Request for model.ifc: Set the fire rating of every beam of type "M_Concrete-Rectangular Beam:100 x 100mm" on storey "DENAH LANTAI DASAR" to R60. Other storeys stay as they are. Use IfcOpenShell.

First a look at what the model holds.

```python
import ifcopenshell
import ifcopenshell.util.element

model = ifcopenshell.open("model.ifc")
print(model.schema)
storey = next(s for s in model.by_type("IfcBuildingStorey") if s.Name == "DENAH LANTAI DASAR")
beams = [e for e in ifcopenshell.util.element.get_decomposition(storey) if e.is_a("IfcBeam")]
seen = {}
for e in beams:
    element_type = ifcopenshell.util.element.get_type(e)
    key = (element_type.Name if element_type != e and element_type else None, ifcopenshell.util.element.get_pset(e, "Pset_BeamCommon", "FireRating"))
    seen[key] = seen.get(key, 0) + 1
for (name, value), count in sorted(seen.items(), key=str):
    print(count, "x", name, "|", value)
```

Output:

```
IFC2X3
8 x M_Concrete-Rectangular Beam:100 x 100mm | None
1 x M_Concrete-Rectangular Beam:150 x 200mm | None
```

```python
import ifcopenshell
import ifcopenshell.api.pset
import ifcopenshell.util.element

model = ifcopenshell.open("model.ifc")

storey = next(s for s in model.by_type("IfcBuildingStorey") if s.Name == "DENAH LANTAI DASAR")
beams = [e for e in ifcopenshell.util.element.get_decomposition(storey) if e.is_a("IfcBeam")]

count = 0
for e in beams:
    element_type = ifcopenshell.util.element.get_type(e)
    if element_type in (None, e) or element_type.Name != "M_Concrete-Rectangular Beam:100 x 100mm":
        continue
    # add_pset returns the element's existing set when there is one.
    pset = ifcopenshell.api.pset.add_pset(model, product=e, name="Pset_BeamCommon")
    ifcopenshell.api.pset.edit_pset(model, pset=pset, properties={"FireRating": "R60"})
    count += 1

print(count, "beams updated")

model.write("model_v2.ifc")
```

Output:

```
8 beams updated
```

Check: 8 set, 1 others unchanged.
